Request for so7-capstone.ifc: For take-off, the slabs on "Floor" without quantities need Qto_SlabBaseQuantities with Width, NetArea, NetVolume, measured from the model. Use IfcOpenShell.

First a look at what the model holds.

```python
import ifcopenshell
import ifcopenshell.util.element
import ifcopenshell.util.unit

model = ifcopenshell.open("so7-capstone.ifc")
print(model.schema)
for unit_type in ("LENGTHUNIT", "AREAUNIT", "VOLUMEUNIT"):
    print(unit_type, ifcopenshell.util.unit.calculate_unit_scale(model, unit_type))
storey = next(s for s in model.by_type("IfcBuildingStorey") if s.Name == "Floor")
slabs = [e for e in ifcopenshell.util.element.get_decomposition(storey) if e.is_a("IfcSlab")]
for e in sorted(slabs, key=lambda e: e.id()):
    print(e.id(), e.is_a(), e.Name, list(ifcopenshell.util.element.get_psets(e, qtos_only=True)), sep=" | ")
```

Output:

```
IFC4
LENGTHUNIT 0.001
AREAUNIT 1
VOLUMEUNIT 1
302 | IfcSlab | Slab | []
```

```python
import ifcopenshell
import ifcopenshell.api.pset
import ifcopenshell.geom
import ifcopenshell.util.element
import ifcopenshell.util.shape
import ifcopenshell.util.unit

model = ifcopenshell.open("so7-capstone.ifc")
unit_scale = ifcopenshell.util.unit.calculate_unit_scale(model)
area_scale = ifcopenshell.util.unit.calculate_unit_scale(model, "AREAUNIT")
volume_scale = ifcopenshell.util.unit.calculate_unit_scale(model, "VOLUMEUNIT")
settings = ifcopenshell.geom.settings()

storey = next(s for s in model.by_type("IfcBuildingStorey") if s.Name == "Floor")
slabs = [e for e in ifcopenshell.util.element.get_decomposition(storey) if e.is_a("IfcSlab")]

for e in sorted(slabs, key=lambda e: e.id()):
    if ifcopenshell.util.element.get_psets(e, qtos_only=True, should_inherit=False):
        continue
    # Geometry comes back in metres, in the element's own axes.
    shape = ifcopenshell.geom.create_shape(settings, e)
    values = {
        "Width": ifcopenshell.util.shape.get_z(shape.geometry) / unit_scale,
        "NetArea": ifcopenshell.util.shape.get_footprint_area(shape.geometry) / area_scale,
        "NetVolume": ifcopenshell.util.shape.get_volume(shape.geometry) / volume_scale,
    }
    qto = ifcopenshell.api.pset.add_qto(model, product=e, name="Qto_SlabBaseQuantities")
    ifcopenshell.api.pset.edit_qto(model, qto=qto, properties=values)
    print(e.id(), {k: round(v, 3) for k, v in values.items()})

model.write("so7-capstone_edited.ifc")
```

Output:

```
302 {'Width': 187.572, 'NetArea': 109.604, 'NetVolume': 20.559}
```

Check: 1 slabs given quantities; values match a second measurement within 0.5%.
